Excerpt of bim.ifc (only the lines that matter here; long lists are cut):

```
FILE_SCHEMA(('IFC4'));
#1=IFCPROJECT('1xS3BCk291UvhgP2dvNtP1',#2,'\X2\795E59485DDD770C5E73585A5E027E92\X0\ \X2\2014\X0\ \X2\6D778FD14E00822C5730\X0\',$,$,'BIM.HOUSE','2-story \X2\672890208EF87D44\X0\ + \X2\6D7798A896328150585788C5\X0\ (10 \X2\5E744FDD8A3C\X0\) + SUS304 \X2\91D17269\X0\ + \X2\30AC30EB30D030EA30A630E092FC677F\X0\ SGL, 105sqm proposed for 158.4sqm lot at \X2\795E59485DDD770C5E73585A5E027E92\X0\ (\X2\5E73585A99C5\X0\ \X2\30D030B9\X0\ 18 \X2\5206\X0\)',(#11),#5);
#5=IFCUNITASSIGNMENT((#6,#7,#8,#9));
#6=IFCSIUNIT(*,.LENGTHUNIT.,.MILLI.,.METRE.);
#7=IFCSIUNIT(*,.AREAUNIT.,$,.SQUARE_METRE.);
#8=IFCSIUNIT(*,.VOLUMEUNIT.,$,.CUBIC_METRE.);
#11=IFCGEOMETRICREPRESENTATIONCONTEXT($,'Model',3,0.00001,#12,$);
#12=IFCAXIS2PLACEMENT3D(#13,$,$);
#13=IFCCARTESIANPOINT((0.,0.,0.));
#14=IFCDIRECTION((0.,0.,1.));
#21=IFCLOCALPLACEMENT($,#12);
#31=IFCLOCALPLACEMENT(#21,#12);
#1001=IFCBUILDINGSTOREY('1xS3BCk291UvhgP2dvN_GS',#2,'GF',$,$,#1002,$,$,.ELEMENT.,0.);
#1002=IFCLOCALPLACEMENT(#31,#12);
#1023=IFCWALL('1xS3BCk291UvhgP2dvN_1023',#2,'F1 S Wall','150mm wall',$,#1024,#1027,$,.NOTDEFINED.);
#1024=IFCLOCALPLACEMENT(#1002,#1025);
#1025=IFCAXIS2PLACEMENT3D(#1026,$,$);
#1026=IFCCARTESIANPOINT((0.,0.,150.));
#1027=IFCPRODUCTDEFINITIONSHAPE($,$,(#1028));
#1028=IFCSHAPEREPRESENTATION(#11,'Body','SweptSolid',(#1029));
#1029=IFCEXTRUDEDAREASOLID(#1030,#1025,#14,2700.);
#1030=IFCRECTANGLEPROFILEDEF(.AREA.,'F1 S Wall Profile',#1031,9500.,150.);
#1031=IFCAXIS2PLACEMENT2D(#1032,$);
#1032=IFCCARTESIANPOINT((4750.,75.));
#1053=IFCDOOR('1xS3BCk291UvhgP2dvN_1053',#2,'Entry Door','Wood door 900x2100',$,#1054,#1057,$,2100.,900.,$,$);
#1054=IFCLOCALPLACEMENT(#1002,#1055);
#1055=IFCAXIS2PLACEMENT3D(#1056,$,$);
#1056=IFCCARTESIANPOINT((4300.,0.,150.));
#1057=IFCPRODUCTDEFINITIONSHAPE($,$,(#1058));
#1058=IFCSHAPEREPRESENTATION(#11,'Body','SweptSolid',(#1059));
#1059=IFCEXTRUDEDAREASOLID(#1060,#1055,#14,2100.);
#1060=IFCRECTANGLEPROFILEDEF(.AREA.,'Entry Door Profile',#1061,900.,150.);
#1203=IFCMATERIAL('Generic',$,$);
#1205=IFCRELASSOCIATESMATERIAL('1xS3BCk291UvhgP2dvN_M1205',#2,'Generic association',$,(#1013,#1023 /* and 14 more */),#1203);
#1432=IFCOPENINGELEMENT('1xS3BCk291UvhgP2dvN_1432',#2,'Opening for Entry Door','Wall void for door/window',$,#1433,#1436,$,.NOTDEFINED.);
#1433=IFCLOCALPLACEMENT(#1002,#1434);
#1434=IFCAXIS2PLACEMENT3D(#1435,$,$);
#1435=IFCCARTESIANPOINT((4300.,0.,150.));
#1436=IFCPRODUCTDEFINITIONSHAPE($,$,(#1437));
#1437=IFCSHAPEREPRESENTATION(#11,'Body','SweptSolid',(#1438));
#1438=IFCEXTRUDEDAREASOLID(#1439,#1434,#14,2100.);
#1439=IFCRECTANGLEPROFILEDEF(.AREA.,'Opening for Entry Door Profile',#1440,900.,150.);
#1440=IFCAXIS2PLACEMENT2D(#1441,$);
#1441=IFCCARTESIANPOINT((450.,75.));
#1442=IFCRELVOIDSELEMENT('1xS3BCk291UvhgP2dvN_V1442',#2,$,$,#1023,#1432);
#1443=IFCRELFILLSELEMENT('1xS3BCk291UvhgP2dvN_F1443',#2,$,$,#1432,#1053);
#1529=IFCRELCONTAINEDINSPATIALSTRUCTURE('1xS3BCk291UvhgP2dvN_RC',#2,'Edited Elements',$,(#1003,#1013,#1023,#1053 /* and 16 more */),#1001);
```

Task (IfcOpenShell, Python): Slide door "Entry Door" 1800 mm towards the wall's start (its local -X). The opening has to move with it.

```python
import ifcopenshell
import ifcopenshell.api.geometry
import ifcopenshell.util.placement

model = ifcopenshell.open("bim.ifc")

door = model.by_guid("1xS3BCk291UvhgP2dvN_1053")
opening = door.FillsVoids[0].RelatingOpeningElement
wall = opening.VoidsElements[0].RelatingBuildingElement

wall_matrix = ifcopenshell.util.placement.get_local_placement(wall.ObjectPlacement)
shift = wall_matrix[:3, 0] * -1800.0
before = ifcopenshell.util.placement.get_local_placement(door.ObjectPlacement)[:3, 3].copy()

# The door is not placed relative to its opening, so move both.
for product in (opening, door):
    matrix = ifcopenshell.util.placement.get_local_placement(product.ObjectPlacement)
    matrix[:3, 3] += shift
    ifcopenshell.api.geometry.edit_object_placement(model, product=product, matrix=matrix, is_si=False)

after = ifcopenshell.util.placement.get_local_placement(door.ObjectPlacement)[:3, 3]
print("door moved by", (after - before).round(3) + 0.0)

model.write("bim_rev.ifc")
```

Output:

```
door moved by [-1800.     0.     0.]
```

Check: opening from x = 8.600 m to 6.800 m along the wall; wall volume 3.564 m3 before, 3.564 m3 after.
